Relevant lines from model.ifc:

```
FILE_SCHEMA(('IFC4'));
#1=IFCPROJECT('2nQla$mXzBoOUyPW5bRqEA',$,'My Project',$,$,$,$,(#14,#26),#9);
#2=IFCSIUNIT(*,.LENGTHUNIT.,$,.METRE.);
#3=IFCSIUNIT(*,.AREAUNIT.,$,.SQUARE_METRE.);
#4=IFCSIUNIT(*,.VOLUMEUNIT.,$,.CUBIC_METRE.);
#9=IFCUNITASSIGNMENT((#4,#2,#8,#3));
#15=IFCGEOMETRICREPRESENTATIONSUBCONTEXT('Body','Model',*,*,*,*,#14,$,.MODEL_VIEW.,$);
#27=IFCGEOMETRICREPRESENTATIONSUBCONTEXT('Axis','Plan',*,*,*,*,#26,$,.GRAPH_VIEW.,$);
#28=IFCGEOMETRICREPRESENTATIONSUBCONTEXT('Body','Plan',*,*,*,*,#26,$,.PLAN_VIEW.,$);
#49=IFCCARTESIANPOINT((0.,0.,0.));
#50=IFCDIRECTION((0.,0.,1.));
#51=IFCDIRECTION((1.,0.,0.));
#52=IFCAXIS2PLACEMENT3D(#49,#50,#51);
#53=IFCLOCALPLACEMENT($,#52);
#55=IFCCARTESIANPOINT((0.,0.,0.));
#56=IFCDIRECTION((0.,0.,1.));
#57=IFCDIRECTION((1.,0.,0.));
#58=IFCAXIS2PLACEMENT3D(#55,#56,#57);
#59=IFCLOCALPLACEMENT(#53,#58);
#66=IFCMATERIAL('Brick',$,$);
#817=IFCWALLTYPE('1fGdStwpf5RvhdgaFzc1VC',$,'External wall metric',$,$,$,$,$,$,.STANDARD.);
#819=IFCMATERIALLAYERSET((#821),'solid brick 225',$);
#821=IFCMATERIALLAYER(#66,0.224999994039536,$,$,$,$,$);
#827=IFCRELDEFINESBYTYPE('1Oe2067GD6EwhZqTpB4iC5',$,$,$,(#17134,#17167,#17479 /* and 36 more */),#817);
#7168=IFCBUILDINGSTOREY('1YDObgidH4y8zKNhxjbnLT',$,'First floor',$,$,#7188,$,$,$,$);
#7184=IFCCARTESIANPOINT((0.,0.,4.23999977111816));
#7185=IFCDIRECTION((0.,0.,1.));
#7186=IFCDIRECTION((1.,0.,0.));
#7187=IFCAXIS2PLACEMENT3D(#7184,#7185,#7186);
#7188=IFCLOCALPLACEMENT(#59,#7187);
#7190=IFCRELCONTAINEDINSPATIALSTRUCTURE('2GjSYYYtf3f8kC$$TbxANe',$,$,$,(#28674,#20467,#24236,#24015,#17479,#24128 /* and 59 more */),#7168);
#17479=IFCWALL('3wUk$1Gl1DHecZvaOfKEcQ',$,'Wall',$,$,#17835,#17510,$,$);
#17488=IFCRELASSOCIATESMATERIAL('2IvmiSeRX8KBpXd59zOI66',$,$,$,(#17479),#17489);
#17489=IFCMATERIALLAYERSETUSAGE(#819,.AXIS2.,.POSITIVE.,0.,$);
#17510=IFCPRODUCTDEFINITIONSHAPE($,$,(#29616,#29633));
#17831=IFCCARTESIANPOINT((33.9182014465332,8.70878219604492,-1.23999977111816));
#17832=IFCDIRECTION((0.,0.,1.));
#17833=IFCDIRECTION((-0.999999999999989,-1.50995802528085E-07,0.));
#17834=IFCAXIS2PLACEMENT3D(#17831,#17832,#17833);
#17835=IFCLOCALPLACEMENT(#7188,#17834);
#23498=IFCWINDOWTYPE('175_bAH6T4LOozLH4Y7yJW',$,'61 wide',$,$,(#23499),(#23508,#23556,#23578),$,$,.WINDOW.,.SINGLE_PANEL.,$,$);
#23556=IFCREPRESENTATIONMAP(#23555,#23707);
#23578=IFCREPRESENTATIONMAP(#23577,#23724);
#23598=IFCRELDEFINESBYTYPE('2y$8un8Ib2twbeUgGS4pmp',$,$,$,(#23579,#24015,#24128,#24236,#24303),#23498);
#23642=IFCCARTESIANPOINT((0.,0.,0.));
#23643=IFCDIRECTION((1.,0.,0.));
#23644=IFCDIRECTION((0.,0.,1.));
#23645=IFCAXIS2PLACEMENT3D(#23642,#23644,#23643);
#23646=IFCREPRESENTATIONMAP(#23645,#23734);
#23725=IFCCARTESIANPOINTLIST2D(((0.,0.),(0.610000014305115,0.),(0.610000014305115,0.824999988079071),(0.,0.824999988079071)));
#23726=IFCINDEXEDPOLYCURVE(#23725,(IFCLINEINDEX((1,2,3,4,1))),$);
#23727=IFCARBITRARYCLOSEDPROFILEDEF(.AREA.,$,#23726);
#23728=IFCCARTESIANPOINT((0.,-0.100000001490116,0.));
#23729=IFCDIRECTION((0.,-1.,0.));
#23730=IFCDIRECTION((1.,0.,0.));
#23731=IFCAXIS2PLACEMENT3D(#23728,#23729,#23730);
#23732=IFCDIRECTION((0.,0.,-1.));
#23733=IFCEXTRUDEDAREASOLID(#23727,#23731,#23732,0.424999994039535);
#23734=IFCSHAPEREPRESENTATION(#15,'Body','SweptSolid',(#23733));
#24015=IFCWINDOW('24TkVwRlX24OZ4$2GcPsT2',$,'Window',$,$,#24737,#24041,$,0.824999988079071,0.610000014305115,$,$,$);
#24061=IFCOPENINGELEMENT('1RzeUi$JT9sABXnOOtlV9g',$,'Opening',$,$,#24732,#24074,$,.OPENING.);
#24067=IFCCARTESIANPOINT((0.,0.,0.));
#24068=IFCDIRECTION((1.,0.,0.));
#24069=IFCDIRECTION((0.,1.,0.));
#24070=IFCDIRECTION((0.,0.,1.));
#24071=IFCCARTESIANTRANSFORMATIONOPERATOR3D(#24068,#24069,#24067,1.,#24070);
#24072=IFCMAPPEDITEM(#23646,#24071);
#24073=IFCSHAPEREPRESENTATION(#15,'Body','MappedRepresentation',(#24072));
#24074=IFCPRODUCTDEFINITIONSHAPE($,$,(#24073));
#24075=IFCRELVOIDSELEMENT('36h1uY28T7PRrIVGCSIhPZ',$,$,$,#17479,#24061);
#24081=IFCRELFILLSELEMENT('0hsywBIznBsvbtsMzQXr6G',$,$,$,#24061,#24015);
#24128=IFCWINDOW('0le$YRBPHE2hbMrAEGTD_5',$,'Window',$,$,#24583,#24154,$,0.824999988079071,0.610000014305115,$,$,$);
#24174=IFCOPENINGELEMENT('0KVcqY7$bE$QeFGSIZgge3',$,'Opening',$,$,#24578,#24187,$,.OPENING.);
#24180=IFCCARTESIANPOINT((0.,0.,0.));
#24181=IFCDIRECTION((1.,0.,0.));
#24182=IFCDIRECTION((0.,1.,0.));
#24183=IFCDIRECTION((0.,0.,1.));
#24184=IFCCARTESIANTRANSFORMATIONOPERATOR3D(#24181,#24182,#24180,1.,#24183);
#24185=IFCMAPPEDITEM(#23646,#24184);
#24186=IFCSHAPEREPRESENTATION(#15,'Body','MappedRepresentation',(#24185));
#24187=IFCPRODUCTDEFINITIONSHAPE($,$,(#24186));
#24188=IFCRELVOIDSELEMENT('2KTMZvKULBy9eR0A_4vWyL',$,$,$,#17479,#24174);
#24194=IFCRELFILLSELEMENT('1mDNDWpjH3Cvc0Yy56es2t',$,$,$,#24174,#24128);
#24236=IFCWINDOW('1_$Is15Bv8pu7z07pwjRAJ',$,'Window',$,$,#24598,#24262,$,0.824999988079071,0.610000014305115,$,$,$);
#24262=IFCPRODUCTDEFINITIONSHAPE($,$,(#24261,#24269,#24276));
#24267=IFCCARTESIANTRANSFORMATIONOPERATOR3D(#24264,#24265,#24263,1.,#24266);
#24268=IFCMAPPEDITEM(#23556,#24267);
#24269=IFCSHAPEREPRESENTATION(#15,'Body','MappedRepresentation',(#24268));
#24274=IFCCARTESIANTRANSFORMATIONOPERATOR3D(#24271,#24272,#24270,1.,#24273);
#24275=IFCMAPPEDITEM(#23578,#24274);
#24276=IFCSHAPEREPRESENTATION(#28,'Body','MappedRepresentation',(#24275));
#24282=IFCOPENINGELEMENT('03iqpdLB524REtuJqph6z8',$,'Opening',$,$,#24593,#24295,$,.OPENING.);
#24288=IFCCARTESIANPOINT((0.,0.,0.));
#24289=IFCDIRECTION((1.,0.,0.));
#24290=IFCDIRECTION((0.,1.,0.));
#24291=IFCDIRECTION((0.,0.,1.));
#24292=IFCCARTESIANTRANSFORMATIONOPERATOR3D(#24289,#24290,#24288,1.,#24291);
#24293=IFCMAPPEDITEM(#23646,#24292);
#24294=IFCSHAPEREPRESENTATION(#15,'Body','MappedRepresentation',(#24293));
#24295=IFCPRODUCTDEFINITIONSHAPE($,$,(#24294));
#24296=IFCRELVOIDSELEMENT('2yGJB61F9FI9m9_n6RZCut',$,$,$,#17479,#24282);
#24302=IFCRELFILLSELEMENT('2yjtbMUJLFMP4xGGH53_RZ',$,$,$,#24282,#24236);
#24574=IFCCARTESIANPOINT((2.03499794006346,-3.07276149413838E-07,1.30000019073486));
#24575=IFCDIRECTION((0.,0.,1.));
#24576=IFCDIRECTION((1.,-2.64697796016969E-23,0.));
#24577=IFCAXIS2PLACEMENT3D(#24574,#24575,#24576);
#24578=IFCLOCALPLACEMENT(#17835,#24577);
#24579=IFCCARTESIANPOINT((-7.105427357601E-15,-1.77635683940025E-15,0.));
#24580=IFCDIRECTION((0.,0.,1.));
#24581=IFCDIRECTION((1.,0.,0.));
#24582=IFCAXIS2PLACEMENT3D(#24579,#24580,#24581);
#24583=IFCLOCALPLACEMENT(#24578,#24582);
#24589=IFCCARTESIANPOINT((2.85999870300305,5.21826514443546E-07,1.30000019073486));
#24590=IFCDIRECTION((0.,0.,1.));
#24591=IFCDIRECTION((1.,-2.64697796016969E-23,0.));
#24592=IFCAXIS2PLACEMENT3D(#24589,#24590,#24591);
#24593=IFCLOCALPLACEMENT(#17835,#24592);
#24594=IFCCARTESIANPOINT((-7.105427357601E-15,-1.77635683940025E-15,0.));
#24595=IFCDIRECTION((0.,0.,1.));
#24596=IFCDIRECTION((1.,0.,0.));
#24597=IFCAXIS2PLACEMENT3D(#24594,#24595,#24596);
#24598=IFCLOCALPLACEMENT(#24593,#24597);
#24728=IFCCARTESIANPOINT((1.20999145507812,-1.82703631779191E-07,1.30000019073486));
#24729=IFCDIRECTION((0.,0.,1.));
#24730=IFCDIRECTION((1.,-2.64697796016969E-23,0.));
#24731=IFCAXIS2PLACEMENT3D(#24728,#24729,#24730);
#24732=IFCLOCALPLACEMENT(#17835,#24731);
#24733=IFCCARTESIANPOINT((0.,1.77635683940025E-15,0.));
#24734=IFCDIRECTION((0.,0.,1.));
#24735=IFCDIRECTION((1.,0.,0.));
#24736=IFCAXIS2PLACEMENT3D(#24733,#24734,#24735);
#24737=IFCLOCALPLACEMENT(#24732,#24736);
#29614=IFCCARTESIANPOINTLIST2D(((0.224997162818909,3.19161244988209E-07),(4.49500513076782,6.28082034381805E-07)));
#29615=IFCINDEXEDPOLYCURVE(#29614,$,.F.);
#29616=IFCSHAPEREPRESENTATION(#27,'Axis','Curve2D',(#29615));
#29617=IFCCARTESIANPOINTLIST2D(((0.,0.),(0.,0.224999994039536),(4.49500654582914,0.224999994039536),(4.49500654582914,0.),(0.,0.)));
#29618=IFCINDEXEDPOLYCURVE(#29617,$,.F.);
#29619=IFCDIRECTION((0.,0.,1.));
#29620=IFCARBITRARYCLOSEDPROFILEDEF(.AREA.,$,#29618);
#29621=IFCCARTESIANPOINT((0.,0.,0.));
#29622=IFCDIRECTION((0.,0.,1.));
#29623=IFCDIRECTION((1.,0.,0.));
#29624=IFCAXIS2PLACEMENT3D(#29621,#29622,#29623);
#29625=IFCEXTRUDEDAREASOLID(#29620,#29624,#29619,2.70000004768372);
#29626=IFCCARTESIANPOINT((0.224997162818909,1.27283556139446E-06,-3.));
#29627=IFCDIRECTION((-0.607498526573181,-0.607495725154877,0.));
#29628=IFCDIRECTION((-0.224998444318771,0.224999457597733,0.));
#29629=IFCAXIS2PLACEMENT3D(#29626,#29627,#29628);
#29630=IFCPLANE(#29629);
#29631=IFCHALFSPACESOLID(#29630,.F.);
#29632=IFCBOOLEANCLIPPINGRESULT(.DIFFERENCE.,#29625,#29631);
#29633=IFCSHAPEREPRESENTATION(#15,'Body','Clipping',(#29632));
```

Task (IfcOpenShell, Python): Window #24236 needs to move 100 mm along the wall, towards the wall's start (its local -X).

```python
import ifcopenshell
import ifcopenshell.api.geometry
import ifcopenshell.util.placement

model = ifcopenshell.open("model.ifc")

window = model.by_id(24236)
opening = window.FillsVoids[0].RelatingOpeningElement
wall = opening.VoidsElements[0].RelatingBuildingElement

wall_matrix = ifcopenshell.util.placement.get_local_placement(wall.ObjectPlacement)
shift = wall_matrix[:3, 0] * -0.1
before = ifcopenshell.util.placement.get_local_placement(window.ObjectPlacement)[:3, 3].copy()

# The window is placed relative to its opening, so it follows when the opening moves.
matrix = ifcopenshell.util.placement.get_local_placement(opening.ObjectPlacement)
matrix[:3, 3] += shift
ifcopenshell.api.geometry.edit_object_placement(
    model, product=opening, matrix=matrix, is_si=False, should_transform_children=True
)

after = ifcopenshell.util.placement.get_local_placement(window.ObjectPlacement)[:3, 3]
print("window moved by", (after - before).round(3) + 0.0)

model.write("model-out.ifc")
```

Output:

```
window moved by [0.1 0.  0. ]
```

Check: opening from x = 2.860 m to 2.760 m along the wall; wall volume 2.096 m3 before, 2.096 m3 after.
